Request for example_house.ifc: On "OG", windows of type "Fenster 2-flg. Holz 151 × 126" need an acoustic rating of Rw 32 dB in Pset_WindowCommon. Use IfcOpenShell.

First a look at what the model holds.

```python
import ifcopenshell
import ifcopenshell.util.element

model = ifcopenshell.open("example_house.ifc")
print(model.schema)
storey = next(s for s in model.by_type("IfcBuildingStorey") if s.Name == "OG")
windows = [e for e in ifcopenshell.util.element.get_decomposition(storey) if e.is_a("IfcWindow")]
seen = {}
for e in windows:
    element_type = ifcopenshell.util.element.get_type(e)
    key = (element_type.Name if element_type != e and element_type else None, ifcopenshell.util.element.get_pset(e, "Pset_WindowCommon", "AcousticRating"))
    seen[key] = seen.get(key, 0) + 1
for (name, value), count in sorted(seen.items(), key=str):
    print(count, "x", name, "|", value)
```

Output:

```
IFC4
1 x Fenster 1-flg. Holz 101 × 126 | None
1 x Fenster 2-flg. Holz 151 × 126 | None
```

```python
import ifcopenshell
import ifcopenshell.api.pset
import ifcopenshell.util.element

model = ifcopenshell.open("example_house.ifc")

storey = next(s for s in model.by_type("IfcBuildingStorey") if s.Name == "OG")
windows = [e for e in ifcopenshell.util.element.get_decomposition(storey) if e.is_a("IfcWindow")]

count = 0
for e in windows:
    element_type = ifcopenshell.util.element.get_type(e)
    if element_type in (None, e) or element_type.Name != "Fenster 2-flg. Holz 151 × 126":
        continue
    # add_pset returns the element's existing set when there is one.
    pset = ifcopenshell.api.pset.add_pset(model, product=e, name="Pset_WindowCommon")
    ifcopenshell.api.pset.edit_pset(model, pset=pset, properties={"AcousticRating": "Rw 32 dB"})
    count += 1

print(count, "windows updated")

model.write("example_house_edited.ifc")
```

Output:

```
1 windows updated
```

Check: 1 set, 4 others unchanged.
